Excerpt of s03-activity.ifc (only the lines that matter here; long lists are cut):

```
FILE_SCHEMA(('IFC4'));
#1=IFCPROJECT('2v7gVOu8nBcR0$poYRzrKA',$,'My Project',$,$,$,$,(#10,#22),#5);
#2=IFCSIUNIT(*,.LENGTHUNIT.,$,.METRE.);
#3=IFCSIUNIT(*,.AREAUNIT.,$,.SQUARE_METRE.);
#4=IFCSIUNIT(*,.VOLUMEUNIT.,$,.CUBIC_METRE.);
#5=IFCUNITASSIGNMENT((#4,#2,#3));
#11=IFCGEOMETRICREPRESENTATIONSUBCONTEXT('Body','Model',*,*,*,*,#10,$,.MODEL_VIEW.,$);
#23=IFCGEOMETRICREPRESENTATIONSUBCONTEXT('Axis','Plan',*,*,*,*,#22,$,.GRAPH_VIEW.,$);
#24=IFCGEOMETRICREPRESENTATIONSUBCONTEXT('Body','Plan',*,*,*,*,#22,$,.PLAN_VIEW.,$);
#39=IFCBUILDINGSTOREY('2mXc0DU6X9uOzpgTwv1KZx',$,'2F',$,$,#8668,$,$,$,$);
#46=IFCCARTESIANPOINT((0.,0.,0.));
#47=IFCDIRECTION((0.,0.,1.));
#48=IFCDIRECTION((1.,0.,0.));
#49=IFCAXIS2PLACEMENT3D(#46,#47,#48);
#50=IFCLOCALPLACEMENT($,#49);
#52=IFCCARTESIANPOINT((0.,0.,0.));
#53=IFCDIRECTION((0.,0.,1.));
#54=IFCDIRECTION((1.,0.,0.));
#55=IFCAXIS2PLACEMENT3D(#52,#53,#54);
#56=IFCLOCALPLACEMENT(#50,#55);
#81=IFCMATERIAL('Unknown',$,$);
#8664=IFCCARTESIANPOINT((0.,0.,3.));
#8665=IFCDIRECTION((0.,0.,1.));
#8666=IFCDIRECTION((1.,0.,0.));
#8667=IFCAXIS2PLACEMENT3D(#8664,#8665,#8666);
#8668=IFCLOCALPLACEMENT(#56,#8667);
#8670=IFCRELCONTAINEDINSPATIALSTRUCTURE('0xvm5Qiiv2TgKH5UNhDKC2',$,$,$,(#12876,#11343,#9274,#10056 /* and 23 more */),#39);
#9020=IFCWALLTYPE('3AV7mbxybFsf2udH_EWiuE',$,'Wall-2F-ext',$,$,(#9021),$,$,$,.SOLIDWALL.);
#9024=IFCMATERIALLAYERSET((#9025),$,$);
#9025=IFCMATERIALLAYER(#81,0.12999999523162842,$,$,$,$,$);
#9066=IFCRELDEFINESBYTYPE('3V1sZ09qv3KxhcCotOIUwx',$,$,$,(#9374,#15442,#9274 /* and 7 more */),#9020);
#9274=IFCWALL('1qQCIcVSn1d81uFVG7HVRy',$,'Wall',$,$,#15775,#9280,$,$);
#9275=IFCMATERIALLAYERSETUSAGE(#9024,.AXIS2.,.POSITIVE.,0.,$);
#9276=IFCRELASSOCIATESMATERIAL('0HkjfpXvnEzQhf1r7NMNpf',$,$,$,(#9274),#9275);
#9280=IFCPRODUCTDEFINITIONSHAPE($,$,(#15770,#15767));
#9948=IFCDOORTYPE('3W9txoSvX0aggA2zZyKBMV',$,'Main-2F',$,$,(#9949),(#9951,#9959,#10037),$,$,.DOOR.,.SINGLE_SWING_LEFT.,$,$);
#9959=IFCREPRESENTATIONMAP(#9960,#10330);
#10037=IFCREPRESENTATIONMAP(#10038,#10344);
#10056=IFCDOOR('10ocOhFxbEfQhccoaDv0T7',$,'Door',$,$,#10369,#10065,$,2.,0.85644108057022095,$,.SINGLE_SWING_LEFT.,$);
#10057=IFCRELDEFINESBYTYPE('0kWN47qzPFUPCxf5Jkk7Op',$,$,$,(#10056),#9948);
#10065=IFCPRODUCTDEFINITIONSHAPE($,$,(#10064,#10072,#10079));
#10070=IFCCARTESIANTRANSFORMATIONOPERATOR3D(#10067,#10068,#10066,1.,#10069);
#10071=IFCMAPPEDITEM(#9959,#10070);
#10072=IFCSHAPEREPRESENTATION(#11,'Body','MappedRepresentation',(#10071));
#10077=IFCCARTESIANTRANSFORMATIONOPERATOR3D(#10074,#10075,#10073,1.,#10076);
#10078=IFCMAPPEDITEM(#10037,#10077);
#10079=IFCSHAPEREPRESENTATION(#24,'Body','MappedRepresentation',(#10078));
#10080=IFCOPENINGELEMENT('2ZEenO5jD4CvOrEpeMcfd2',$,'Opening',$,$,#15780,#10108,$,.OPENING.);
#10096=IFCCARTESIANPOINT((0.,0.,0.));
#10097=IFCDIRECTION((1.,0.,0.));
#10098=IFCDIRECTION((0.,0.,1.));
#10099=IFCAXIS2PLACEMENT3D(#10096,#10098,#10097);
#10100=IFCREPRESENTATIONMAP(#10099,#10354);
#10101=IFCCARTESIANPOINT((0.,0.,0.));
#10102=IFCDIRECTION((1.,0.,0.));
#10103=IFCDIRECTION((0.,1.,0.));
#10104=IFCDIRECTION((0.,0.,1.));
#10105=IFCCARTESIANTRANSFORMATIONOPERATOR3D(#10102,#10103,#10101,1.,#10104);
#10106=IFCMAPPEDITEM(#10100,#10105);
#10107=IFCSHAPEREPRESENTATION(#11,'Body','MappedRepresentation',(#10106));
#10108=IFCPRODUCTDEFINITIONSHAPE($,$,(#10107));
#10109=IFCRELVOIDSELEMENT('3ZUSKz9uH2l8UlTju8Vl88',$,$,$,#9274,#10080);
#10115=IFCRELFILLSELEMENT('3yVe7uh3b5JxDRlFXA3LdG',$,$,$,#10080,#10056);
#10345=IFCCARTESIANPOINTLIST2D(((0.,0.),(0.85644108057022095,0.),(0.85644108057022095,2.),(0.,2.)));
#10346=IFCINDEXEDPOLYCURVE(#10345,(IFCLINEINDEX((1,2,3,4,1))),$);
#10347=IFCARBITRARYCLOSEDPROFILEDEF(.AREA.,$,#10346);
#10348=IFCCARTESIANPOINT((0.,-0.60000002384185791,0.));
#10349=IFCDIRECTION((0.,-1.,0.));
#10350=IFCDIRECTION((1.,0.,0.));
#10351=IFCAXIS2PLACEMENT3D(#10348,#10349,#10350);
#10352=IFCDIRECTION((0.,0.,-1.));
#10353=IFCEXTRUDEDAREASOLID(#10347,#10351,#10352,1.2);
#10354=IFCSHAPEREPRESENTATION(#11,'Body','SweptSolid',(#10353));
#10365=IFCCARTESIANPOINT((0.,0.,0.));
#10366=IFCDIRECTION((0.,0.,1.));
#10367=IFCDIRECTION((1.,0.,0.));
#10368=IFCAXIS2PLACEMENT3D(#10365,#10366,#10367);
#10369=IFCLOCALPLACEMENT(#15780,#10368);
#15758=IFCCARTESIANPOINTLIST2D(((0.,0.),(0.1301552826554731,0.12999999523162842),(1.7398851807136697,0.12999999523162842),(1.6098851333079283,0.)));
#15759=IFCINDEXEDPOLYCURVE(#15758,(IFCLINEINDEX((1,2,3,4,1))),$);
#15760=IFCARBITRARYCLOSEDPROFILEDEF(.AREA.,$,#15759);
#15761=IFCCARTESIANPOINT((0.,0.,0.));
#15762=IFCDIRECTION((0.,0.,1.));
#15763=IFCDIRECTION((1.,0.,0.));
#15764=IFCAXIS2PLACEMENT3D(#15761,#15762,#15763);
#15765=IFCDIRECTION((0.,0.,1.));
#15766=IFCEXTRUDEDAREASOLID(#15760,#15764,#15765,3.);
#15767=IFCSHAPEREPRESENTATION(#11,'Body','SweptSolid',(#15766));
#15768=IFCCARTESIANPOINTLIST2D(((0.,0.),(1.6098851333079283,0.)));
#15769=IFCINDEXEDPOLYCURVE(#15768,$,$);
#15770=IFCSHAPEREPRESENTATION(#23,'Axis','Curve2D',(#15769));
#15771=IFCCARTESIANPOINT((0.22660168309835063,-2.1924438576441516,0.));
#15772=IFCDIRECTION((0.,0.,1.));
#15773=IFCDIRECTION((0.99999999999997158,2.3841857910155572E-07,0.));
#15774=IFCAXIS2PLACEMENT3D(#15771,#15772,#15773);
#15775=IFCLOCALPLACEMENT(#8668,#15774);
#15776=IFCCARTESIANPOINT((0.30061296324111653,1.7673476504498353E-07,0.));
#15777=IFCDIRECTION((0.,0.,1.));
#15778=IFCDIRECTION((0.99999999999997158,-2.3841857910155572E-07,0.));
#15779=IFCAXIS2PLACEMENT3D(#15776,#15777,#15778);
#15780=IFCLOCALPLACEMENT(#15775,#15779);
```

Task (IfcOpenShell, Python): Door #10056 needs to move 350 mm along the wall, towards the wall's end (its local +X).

```python
import ifcopenshell
import ifcopenshell.api.geometry
import ifcopenshell.util.placement
import ifcopenshell.util.unit

model = ifcopenshell.open("s03-activity.ifc")
unit_scale = ifcopenshell.util.unit.calculate_unit_scale(model)

door = model.by_id(10056)
opening = door.FillsVoids[0].RelatingOpeningElement
wall = opening.VoidsElements[0].RelatingBuildingElement

wall_matrix = ifcopenshell.util.placement.get_local_placement(wall.ObjectPlacement)
shift = wall_matrix[:3, 0] * 0.35 / unit_scale
before = ifcopenshell.util.placement.get_local_placement(door.ObjectPlacement)[:3, 3].copy()

# The door is placed relative to its opening, so it follows when the opening moves.
matrix = ifcopenshell.util.placement.get_local_placement(opening.ObjectPlacement)
matrix[:3, 3] += shift
ifcopenshell.api.geometry.edit_object_placement(
    model, product=opening, matrix=matrix, is_si=False, should_transform_children=True
)

after = ifcopenshell.util.placement.get_local_placement(door.ObjectPlacement)[:3, 3]
print("door moved by", (after - before).round(3) + 0.0)

model.write("s03-activity_v2.ifc")
```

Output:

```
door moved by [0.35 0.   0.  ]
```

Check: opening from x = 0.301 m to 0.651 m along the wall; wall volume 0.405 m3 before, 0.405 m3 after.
